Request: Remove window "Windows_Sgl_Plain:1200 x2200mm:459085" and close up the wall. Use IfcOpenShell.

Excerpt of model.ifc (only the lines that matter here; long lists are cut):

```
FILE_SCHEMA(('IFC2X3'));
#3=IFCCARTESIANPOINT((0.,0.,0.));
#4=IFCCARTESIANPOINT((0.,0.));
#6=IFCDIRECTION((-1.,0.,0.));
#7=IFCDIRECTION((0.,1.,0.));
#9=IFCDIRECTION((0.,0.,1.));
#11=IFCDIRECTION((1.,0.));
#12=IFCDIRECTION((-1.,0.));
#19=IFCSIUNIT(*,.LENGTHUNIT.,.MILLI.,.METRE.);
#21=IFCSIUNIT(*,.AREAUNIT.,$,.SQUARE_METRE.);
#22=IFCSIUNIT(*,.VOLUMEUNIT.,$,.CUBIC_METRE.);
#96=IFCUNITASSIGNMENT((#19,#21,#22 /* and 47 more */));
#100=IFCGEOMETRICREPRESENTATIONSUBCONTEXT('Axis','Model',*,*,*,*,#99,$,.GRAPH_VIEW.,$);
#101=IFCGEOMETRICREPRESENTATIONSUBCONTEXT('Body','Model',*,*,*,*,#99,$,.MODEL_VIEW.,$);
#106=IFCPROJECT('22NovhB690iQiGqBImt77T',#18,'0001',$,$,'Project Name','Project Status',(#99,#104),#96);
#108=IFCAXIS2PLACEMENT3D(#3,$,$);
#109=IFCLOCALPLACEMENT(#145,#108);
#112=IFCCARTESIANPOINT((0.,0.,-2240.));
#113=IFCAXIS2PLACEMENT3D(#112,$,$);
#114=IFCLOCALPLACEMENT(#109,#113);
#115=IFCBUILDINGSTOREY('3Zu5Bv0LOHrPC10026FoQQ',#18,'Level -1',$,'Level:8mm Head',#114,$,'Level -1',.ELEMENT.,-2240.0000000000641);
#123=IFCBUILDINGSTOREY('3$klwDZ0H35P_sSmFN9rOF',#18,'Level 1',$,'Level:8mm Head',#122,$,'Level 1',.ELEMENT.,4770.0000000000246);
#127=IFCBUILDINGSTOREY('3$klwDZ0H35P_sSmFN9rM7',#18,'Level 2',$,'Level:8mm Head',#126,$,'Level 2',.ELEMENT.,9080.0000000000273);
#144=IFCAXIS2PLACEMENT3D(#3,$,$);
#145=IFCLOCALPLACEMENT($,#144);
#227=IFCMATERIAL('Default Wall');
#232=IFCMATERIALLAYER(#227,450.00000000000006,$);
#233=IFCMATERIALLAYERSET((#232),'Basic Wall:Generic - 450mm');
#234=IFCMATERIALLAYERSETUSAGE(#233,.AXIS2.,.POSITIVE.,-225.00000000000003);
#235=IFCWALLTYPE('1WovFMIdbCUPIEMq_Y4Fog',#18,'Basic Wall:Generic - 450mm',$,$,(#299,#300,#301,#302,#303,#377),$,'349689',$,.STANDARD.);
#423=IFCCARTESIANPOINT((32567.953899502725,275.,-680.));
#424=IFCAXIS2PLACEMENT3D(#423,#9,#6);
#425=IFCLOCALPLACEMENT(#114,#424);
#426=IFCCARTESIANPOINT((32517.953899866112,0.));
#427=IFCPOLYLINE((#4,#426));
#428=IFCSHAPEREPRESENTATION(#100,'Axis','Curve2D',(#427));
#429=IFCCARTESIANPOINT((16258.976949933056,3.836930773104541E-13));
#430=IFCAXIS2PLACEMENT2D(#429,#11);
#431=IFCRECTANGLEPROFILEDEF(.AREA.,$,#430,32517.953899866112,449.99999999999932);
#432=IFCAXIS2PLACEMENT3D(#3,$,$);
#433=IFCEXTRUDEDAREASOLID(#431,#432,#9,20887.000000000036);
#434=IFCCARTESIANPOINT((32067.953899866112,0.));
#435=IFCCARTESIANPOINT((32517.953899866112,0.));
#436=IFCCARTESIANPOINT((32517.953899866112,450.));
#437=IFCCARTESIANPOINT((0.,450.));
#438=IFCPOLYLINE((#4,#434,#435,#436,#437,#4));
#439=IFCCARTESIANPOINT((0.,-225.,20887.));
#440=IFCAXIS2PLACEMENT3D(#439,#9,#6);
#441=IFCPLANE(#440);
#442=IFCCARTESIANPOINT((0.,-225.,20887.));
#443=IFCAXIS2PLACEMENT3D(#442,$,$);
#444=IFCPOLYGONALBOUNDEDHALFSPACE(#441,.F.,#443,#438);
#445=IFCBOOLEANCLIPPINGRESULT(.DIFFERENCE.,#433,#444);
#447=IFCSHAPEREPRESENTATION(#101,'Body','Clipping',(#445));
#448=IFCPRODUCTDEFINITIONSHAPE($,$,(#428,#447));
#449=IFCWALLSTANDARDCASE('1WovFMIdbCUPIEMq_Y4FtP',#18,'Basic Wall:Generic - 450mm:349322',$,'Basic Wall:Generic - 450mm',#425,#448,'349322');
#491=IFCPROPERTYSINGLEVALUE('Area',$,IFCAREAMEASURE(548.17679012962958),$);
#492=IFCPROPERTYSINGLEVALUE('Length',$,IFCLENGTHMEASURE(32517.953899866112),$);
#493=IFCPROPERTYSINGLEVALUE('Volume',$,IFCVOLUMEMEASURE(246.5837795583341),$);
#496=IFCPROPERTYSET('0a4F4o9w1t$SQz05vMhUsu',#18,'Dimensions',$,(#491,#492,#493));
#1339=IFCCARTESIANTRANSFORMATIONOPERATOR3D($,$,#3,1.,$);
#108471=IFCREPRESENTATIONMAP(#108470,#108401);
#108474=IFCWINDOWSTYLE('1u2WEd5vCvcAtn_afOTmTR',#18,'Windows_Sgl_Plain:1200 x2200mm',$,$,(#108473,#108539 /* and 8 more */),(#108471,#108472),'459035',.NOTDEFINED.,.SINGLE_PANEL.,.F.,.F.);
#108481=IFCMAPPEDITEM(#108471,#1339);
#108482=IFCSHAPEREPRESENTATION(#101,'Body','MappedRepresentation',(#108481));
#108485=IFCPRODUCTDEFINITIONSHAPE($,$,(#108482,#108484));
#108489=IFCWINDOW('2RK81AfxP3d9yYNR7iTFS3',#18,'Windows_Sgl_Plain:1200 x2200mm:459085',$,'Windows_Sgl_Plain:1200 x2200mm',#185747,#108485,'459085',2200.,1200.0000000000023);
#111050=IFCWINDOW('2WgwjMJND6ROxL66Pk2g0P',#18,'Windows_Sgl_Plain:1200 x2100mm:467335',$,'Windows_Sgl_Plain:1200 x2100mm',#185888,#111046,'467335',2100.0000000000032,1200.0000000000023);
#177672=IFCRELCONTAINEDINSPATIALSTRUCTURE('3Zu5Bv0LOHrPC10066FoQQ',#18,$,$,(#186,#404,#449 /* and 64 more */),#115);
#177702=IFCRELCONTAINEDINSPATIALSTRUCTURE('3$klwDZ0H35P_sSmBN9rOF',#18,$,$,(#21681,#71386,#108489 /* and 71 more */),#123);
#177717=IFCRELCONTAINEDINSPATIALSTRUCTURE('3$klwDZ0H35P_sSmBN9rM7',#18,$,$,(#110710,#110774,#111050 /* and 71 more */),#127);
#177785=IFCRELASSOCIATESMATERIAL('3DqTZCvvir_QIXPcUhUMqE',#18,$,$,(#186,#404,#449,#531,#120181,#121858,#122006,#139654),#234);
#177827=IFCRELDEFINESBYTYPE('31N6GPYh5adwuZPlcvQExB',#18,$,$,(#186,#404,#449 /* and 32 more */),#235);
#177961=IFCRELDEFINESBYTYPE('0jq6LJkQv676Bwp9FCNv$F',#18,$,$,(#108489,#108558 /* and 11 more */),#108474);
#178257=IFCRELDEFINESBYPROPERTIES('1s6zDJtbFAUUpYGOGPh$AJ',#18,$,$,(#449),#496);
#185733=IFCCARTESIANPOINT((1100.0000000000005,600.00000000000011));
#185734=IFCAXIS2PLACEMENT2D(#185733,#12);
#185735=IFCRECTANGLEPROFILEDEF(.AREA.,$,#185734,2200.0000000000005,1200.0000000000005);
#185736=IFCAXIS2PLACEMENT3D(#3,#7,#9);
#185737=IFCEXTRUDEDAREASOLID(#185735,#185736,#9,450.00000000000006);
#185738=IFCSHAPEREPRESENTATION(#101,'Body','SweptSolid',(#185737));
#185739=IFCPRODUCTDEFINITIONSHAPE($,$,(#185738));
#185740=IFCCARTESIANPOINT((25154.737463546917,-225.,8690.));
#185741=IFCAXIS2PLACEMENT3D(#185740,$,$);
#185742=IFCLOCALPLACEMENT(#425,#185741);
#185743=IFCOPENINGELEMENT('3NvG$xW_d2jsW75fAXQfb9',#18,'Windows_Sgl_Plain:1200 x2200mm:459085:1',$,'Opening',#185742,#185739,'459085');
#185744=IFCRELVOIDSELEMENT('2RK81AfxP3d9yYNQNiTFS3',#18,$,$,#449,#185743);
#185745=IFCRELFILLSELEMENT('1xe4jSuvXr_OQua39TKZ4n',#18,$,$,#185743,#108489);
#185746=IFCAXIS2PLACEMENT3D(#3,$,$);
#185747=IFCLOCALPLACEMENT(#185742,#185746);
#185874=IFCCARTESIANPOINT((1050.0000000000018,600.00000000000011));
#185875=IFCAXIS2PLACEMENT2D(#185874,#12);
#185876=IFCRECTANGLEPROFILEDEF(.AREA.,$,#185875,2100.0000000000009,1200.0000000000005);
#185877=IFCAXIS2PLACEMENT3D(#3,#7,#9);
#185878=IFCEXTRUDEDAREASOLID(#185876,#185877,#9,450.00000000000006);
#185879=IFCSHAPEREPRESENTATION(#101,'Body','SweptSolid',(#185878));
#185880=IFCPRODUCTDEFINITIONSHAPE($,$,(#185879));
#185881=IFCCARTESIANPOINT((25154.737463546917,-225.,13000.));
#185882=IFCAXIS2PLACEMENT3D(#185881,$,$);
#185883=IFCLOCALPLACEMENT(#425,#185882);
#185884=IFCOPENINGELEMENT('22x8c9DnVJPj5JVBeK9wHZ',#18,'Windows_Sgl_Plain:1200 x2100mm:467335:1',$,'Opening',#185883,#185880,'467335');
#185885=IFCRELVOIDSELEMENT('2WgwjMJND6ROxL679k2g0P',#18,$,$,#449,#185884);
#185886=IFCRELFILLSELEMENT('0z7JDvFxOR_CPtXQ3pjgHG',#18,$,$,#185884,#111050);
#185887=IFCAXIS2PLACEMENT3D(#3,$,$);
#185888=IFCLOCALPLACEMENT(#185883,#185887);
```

```python
import ifcopenshell
import ifcopenshell.api.feature
import ifcopenshell.api.pset
import ifcopenshell.api.root
import ifcopenshell.geom
import ifcopenshell.util.element
import ifcopenshell.util.shape
import ifcopenshell.util.unit

model = ifcopenshell.open("model.ifc")
area_scale = ifcopenshell.util.unit.calculate_unit_scale(model, "AREAUNIT")
volume_scale = ifcopenshell.util.unit.calculate_unit_scale(model, "VOLUMEUNIT")
settings = ifcopenshell.geom.settings()


def volume(element):
    """Net volume in cubic metres, openings subtracted."""
    shape = ifcopenshell.geom.create_shape(settings, element)
    return ifcopenshell.util.shape.get_volume(shape.geometry)


window = model.by_guid("2RK81AfxP3d9yYNR7iTFS3")
opening = window.FillsVoids[0].RelatingOpeningElement
wall = opening.VoidsElements[0].RelatingBuildingElement
before = volume(wall)

ifcopenshell.api.root.remove_product(model, product=window)
ifcopenshell.api.feature.remove_feature(model, feature=opening)

after = volume(wall)
thickness = 0.45  # wall thickness in metres

# Update the wall's stored quantities.
pset = model.by_id(ifcopenshell.util.element.get_pset(wall, "Dimensions", should_inherit=False)["id"])
ifcopenshell.api.pset.edit_pset(model, pset=pset, properties={
    "Area": model.create_entity("IfcAreaMeasure", after / thickness / area_scale),
    "Volume": model.create_entity("IfcVolumeMeasure", after / volume_scale),
})

print(f"wall volume {before:.3f} -> {after:.3f} m3")

model.write("model-out.ifc")
```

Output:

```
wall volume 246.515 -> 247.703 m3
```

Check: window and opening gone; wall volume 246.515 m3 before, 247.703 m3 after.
